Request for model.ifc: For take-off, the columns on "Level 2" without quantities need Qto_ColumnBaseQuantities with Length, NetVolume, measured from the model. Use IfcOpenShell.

First a look at what the model holds.

```python
import ifcopenshell
import ifcopenshell.util.element
import ifcopenshell.util.unit

model = ifcopenshell.open("model.ifc")
print(model.schema)
for unit_type in ("LENGTHUNIT", "AREAUNIT", "VOLUMEUNIT"):
    print(unit_type, ifcopenshell.util.unit.calculate_unit_scale(model, unit_type))
storey = next(s for s in model.by_type("IfcBuildingStorey") if s.Name == "Level 2")
columns = [e for e in ifcopenshell.util.element.get_decomposition(storey) if e.is_a("IfcColumn")]
for e in sorted(columns, key=lambda e: e.id()):
    print(e.id(), e.is_a(), e.Name, list(ifcopenshell.util.element.get_psets(e, qtos_only=True)), sep=" | ")
```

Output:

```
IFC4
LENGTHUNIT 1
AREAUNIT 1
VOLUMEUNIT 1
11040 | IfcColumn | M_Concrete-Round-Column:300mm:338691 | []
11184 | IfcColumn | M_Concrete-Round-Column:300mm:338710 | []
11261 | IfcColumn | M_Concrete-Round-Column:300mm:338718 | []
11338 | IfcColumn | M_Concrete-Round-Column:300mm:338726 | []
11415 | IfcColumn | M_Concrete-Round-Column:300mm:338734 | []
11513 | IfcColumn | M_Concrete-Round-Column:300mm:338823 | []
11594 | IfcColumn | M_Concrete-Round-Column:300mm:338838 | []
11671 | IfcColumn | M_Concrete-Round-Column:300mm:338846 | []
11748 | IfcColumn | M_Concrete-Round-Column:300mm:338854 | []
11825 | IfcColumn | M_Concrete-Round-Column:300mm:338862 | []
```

```python
import ifcopenshell
import ifcopenshell.api.pset
import ifcopenshell.geom
import ifcopenshell.util.element
import ifcopenshell.util.shape
import ifcopenshell.util.unit

model = ifcopenshell.open("model.ifc")
unit_scale = ifcopenshell.util.unit.calculate_unit_scale(model)
volume_scale = ifcopenshell.util.unit.calculate_unit_scale(model, "VOLUMEUNIT")
settings = ifcopenshell.geom.settings()

storey = next(s for s in model.by_type("IfcBuildingStorey") if s.Name == "Level 2")
columns = [e for e in ifcopenshell.util.element.get_decomposition(storey) if e.is_a("IfcColumn")]

for e in sorted(columns, key=lambda e: e.id()):
    if ifcopenshell.util.element.get_psets(e, qtos_only=True, should_inherit=False):
        continue
    # Geometry comes back in metres, in the element's own axes.
    shape = ifcopenshell.geom.create_shape(settings, e)
    values = {
        "Length": ifcopenshell.util.shape.get_z(shape.geometry) / unit_scale,
        "NetVolume": ifcopenshell.util.shape.get_volume(shape.geometry) / volume_scale,
    }
    qto = ifcopenshell.api.pset.add_qto(model, product=e, name="Qto_ColumnBaseQuantities")
    ifcopenshell.api.pset.edit_qto(model, qto=qto, properties=values)
    print(e.id(), {k: round(v, 3) for k, v in values.items()})

model.write("model_rev.ifc")
```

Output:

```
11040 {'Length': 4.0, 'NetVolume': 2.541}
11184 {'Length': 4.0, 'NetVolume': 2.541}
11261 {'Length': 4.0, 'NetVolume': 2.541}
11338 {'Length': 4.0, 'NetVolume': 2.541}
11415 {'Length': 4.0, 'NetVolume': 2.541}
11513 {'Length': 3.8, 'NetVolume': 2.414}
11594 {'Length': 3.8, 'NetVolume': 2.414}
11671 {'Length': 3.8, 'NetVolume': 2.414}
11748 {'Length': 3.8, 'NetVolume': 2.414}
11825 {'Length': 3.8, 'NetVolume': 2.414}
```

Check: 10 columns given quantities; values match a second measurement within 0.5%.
